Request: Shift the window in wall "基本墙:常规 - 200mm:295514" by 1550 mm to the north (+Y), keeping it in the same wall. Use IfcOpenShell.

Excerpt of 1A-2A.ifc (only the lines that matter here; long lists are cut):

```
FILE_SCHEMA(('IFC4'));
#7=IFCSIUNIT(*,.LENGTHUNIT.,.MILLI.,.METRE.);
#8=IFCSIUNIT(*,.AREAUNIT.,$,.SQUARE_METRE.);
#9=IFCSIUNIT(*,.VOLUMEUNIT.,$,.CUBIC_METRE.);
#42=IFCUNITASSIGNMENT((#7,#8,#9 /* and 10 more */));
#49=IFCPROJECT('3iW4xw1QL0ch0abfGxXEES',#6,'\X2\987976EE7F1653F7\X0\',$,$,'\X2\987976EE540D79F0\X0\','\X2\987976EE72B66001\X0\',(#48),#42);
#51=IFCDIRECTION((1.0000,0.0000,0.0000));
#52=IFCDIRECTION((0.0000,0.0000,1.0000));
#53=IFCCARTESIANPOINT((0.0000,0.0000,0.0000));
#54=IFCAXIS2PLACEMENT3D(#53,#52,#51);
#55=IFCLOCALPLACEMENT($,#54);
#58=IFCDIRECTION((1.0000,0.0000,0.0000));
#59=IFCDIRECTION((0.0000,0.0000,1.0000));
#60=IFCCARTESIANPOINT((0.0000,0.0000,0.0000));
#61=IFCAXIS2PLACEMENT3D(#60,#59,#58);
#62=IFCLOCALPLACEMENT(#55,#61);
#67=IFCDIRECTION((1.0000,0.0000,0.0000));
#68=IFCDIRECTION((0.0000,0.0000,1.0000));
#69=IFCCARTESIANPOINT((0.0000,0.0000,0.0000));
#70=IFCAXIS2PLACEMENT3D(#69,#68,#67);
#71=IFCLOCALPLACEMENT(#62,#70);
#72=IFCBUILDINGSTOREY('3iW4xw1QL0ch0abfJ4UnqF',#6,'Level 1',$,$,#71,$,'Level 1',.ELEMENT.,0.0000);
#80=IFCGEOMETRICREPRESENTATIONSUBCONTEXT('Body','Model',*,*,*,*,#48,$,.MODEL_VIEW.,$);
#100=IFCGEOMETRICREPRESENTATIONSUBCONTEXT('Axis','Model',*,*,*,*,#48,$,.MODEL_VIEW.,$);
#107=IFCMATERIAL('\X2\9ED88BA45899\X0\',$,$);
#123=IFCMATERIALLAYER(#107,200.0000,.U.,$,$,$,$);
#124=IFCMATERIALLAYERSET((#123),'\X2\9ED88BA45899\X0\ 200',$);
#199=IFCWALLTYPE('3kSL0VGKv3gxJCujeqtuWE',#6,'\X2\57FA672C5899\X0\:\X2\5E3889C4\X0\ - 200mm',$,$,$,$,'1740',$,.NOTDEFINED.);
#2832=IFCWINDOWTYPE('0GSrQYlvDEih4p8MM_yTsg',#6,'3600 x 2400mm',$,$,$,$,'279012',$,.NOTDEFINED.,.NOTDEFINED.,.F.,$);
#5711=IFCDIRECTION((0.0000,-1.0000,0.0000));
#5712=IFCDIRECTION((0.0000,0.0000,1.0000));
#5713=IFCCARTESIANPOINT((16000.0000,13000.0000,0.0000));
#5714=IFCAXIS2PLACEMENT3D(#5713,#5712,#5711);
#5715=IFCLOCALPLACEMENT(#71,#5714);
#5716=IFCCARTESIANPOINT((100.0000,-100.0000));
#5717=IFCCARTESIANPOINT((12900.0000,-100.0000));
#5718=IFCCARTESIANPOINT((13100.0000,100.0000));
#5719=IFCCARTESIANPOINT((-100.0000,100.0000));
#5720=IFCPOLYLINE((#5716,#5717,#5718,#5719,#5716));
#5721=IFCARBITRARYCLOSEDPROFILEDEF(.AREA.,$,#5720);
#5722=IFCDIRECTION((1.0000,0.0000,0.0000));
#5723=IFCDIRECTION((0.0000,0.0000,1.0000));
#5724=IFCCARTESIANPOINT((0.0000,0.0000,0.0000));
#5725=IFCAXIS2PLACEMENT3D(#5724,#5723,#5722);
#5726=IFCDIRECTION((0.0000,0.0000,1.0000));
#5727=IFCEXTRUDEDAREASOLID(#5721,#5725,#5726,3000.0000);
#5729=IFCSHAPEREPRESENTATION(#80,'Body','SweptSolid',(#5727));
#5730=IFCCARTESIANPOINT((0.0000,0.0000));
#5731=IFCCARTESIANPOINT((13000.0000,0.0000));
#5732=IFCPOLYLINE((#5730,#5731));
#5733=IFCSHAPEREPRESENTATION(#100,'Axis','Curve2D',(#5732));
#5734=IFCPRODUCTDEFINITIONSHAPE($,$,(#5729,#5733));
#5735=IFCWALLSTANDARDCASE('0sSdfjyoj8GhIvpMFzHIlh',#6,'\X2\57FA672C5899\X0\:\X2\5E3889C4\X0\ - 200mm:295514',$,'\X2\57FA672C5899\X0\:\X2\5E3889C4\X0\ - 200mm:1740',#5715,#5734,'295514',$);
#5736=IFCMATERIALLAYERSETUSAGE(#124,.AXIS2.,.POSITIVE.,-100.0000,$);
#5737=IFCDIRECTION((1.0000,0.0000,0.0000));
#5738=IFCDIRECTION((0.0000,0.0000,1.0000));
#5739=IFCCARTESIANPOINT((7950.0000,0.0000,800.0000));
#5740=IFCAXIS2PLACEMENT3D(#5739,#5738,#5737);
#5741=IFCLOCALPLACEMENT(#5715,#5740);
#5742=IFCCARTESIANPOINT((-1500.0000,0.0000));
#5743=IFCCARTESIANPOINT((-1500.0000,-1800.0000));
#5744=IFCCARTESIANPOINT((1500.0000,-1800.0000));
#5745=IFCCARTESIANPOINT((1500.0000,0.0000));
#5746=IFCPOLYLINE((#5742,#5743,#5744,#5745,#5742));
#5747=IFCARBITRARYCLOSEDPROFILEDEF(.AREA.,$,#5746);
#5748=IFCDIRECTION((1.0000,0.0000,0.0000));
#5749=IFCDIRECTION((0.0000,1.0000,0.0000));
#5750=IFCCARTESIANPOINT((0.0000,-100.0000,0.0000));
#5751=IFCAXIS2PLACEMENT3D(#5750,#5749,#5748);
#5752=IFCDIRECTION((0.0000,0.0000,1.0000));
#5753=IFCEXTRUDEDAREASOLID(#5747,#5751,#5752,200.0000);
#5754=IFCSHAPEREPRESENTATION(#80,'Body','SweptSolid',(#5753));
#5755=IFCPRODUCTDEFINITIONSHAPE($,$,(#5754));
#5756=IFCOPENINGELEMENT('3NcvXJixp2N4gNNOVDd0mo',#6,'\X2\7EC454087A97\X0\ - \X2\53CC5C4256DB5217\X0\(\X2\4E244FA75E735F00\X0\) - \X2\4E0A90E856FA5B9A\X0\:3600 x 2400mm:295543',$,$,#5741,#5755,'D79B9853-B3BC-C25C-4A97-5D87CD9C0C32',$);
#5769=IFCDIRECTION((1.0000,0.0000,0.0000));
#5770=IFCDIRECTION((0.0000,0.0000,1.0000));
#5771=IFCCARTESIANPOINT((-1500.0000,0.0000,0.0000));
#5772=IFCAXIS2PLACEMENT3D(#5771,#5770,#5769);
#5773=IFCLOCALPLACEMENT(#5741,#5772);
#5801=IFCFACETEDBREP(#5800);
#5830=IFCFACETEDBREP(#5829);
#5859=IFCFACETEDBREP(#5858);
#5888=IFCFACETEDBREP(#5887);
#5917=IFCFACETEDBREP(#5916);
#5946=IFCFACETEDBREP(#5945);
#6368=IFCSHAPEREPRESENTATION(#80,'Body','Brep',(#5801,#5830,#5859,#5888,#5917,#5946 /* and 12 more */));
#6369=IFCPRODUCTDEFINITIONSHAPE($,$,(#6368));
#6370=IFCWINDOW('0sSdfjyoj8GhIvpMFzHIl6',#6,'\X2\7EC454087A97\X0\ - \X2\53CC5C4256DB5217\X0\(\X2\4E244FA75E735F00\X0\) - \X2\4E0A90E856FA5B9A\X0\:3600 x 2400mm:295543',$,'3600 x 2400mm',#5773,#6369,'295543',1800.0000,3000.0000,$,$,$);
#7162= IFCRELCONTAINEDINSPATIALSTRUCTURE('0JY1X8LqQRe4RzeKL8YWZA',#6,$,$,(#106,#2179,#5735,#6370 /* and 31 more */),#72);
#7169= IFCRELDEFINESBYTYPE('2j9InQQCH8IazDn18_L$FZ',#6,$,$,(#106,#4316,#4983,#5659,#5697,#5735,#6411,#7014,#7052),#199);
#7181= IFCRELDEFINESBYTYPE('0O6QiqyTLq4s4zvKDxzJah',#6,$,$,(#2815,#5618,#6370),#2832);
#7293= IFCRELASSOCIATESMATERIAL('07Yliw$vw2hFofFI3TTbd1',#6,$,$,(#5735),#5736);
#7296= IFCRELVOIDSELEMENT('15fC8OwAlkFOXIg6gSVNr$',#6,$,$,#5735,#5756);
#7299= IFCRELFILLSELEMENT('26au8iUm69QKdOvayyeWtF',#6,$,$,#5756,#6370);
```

```python
import ifcopenshell
import ifcopenshell.api.geometry
import ifcopenshell.util.placement
import ifcopenshell.util.unit

model = ifcopenshell.open("1A-2A.ifc")
unit_scale = ifcopenshell.util.unit.calculate_unit_scale(model)

window = model.by_guid("0sSdfjyoj8GhIvpMFzHIl6")
opening = window.FillsVoids[0].RelatingOpeningElement
wall = opening.VoidsElements[0].RelatingBuildingElement

wall_matrix = ifcopenshell.util.placement.get_local_placement(wall.ObjectPlacement)
shift = wall_matrix[:3, 0] * -1.55 / unit_scale
before = ifcopenshell.util.placement.get_local_placement(window.ObjectPlacement)[:3, 3].copy()

# The window is placed relative to its opening, so it follows when the opening moves.
matrix = ifcopenshell.util.placement.get_local_placement(opening.ObjectPlacement)
matrix[:3, 3] += shift
ifcopenshell.api.geometry.edit_object_placement(
    model, product=opening, matrix=matrix, is_si=False, should_transform_children=True
)

after = ifcopenshell.util.placement.get_local_placement(window.ObjectPlacement)[:3, 3]
print("window moved by", (after - before).round(3) + 0.0)

model.write("1A-2A_updated.ifc")
```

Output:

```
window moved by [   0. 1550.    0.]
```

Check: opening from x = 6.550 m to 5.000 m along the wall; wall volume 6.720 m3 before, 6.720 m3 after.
